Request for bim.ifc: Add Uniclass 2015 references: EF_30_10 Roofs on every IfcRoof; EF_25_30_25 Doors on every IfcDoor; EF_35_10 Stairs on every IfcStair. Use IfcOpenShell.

First a look at what the model holds.

```python
import ifcopenshell

model = ifcopenshell.open("bim.ifc")
print(model.schema)
print("classifications:", [c.Name for c in model.by_type("IfcClassification")])
for ifc_class in ("IfcDoor", "IfcRoof", "IfcStair", "IfcWall", "IfcWindow"):
    print(ifc_class, len(model.by_type(ifc_class)))
```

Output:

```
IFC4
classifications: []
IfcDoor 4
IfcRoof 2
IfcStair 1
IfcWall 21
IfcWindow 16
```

```python
import ifcopenshell
import ifcopenshell.api.classification

model = ifcopenshell.open("bim.ifc")

system = ifcopenshell.api.classification.add_classification(model, classification="Uniclass 2015")

codes = {
    "IfcRoof": ("EF_30_10", "Roofs"),
    "IfcDoor": ("EF_25_30_25", "Doors"),
    "IfcStair": ("EF_35_10", "Stairs"),
}
for ifc_class, (code, name) in codes.items():
    products = model.by_type(ifc_class)
    ifcopenshell.api.classification.add_reference(
        model, products=products, classification=system, identification=code, name=name
    )
    print(code, len(products))

model.write("bim_updated.ifc")
```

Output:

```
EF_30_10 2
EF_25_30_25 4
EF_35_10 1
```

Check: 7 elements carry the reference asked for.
